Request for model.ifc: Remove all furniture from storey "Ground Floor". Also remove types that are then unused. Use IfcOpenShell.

First a look at what the model holds.

```python
import ifcopenshell
import ifcopenshell.util.element

model = ifcopenshell.open("model.ifc")
print(model.schema)
storey = next(s for s in model.by_type("IfcBuildingStorey") if s.Name == "Ground Floor")
furniture = [e for e in ifcopenshell.util.element.get_decomposition(storey) if e.is_a("IfcFurnishingElement")]
seen = {}
for e in furniture:
    element_type = ifcopenshell.util.element.get_type(e)
    name = element_type.Name if element_type not in (None, e) else None
    seen[name] = seen.get(name, 0) + 1
for name, count in sorted(seen.items(), key=str):
    print(count, "x", name)
```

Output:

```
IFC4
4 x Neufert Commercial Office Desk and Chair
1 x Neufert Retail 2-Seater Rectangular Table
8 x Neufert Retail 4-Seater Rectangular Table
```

```python
import ifcopenshell
import ifcopenshell.api.root
import ifcopenshell.util.element

model = ifcopenshell.open("model.ifc")

storey = next(s for s in model.by_type("IfcBuildingStorey") if s.Name == "Ground Floor")
furniture = [e for e in ifcopenshell.util.element.get_decomposition(storey) if e.is_a("IfcFurnishingElement")]
types = {ifcopenshell.util.element.get_type(e) for e in furniture} - {None, *furniture}

for e in furniture:
    ifcopenshell.api.root.remove_product(model, product=e)
print(len(furniture), "removed")

unused = [t for t in types if not ifcopenshell.util.element.get_types(t)]
for t in unused:
    ifcopenshell.api.root.remove_product(model, product=t)
print(len(unused), "unused types removed")

model.write("model_rev.ifc")
```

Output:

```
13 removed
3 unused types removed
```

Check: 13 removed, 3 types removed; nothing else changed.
